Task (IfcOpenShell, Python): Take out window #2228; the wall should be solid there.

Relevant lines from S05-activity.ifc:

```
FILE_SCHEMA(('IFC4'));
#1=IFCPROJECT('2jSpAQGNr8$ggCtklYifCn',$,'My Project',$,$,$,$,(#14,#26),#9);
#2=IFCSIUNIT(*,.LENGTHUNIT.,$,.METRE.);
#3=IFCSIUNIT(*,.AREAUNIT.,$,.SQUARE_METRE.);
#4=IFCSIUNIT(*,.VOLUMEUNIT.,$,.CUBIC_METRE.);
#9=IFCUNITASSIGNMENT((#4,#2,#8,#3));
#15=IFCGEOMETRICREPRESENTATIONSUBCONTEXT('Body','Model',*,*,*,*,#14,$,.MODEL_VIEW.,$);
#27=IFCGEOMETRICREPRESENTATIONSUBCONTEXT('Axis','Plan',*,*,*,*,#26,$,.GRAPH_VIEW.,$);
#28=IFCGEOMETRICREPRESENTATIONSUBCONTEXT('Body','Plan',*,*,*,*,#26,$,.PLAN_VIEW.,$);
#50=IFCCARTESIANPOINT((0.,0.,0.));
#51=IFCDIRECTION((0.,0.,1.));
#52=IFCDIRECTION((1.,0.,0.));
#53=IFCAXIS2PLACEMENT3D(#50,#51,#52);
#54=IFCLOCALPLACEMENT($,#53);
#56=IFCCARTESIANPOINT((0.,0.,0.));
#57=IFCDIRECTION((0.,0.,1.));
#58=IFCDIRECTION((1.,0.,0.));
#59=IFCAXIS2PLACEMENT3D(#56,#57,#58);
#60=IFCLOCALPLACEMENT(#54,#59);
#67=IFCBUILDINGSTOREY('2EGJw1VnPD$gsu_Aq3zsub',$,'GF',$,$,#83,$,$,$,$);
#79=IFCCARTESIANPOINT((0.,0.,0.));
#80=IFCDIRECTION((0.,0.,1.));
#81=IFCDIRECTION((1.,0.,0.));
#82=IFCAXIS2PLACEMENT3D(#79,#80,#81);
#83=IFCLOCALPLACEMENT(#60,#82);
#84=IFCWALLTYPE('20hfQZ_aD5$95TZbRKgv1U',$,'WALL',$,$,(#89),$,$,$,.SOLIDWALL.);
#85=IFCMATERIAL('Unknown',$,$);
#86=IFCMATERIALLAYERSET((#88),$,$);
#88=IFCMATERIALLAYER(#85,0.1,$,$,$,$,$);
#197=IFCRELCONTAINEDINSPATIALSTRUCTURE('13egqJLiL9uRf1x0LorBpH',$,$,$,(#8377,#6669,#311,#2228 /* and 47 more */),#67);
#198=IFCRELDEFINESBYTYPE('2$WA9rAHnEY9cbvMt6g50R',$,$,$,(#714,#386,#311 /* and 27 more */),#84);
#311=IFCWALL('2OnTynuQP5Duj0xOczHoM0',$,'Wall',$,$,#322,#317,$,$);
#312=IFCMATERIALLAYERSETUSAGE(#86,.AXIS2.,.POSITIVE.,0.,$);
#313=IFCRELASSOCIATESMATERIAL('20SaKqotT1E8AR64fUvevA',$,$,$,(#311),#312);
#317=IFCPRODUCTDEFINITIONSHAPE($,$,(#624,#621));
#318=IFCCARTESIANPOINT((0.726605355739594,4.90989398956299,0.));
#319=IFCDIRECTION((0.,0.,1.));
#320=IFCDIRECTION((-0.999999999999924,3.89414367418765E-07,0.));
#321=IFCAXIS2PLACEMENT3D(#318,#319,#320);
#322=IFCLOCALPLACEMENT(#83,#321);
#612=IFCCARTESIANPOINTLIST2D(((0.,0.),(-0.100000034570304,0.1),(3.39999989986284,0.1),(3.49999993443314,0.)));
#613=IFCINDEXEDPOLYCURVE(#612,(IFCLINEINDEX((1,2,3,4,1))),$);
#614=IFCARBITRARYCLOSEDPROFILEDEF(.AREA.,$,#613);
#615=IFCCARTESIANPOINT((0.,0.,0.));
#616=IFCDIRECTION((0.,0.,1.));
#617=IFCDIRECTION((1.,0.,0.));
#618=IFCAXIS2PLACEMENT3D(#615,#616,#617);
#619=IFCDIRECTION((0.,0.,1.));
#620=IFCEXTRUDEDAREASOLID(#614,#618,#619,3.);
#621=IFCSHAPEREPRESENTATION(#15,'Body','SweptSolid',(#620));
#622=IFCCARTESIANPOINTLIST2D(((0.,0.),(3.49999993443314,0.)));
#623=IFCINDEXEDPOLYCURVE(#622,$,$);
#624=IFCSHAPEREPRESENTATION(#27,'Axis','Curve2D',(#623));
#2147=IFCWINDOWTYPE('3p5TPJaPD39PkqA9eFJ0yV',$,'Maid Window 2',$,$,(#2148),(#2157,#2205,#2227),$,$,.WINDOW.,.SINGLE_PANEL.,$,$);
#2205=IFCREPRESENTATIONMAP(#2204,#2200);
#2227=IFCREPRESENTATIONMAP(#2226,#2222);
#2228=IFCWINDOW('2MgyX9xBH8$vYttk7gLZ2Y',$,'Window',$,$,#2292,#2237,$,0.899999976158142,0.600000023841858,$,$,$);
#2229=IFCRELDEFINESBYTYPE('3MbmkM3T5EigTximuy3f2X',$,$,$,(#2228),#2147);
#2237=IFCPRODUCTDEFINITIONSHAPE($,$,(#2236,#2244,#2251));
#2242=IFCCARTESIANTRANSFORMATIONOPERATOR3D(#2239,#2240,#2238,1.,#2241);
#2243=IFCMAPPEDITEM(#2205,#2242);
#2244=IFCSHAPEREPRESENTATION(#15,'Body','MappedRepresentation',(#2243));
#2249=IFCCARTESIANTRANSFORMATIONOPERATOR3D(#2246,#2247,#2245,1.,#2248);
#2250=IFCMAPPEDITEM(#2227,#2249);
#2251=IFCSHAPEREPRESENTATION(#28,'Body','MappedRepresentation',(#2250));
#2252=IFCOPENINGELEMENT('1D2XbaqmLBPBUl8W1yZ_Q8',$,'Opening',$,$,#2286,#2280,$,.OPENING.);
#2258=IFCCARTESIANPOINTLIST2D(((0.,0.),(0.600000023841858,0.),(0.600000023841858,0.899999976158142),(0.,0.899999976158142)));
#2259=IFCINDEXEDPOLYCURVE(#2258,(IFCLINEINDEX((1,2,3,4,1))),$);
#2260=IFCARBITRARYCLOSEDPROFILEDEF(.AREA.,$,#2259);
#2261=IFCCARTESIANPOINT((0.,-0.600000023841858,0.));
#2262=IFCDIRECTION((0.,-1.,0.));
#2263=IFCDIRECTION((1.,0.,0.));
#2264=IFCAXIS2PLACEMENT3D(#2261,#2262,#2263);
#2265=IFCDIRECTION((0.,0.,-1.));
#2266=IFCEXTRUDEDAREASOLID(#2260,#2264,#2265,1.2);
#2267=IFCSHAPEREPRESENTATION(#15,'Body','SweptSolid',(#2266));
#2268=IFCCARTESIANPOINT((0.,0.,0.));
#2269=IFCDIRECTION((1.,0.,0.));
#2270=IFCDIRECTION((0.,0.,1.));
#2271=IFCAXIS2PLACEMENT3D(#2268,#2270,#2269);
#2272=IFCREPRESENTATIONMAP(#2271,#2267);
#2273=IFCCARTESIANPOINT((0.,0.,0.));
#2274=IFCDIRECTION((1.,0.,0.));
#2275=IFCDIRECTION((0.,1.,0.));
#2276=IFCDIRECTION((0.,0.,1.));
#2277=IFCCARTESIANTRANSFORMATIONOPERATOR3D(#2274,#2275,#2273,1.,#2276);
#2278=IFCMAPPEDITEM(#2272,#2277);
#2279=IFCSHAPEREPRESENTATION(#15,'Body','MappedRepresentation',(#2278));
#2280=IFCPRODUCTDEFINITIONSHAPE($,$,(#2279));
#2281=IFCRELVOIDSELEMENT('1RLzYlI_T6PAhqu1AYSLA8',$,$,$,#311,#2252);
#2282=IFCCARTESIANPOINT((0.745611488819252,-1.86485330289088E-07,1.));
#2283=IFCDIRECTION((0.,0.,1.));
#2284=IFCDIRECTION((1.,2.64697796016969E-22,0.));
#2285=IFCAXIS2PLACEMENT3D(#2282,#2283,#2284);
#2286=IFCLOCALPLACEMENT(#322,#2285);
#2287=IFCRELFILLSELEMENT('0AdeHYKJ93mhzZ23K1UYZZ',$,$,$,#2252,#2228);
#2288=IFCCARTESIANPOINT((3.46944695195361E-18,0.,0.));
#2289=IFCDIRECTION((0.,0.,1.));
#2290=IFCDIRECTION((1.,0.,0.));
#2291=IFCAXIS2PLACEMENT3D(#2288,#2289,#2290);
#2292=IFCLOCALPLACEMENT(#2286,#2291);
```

```python
import ifcopenshell
import ifcopenshell.api.feature
import ifcopenshell.api.root
import ifcopenshell.geom
import ifcopenshell.util.shape

model = ifcopenshell.open("S05-activity.ifc")
settings = ifcopenshell.geom.settings()


def volume(element):
    """Net volume in cubic metres, openings subtracted."""
    shape = ifcopenshell.geom.create_shape(settings, element)
    return ifcopenshell.util.shape.get_volume(shape.geometry)


window = model.by_guid("2MgyX9xBH8$vYttk7gLZ2Y")
opening = window.FillsVoids[0].RelatingOpeningElement
wall = opening.VoidsElements[0].RelatingBuildingElement
before = volume(wall)

ifcopenshell.api.root.remove_product(model, product=window)
ifcopenshell.api.feature.remove_feature(model, feature=opening)

after = volume(wall)

print(f"wall volume {before:.3f} -> {after:.3f} m3")

model.write("S05-activity-out.ifc")
```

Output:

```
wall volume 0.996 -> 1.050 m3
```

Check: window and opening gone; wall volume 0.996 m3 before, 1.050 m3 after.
